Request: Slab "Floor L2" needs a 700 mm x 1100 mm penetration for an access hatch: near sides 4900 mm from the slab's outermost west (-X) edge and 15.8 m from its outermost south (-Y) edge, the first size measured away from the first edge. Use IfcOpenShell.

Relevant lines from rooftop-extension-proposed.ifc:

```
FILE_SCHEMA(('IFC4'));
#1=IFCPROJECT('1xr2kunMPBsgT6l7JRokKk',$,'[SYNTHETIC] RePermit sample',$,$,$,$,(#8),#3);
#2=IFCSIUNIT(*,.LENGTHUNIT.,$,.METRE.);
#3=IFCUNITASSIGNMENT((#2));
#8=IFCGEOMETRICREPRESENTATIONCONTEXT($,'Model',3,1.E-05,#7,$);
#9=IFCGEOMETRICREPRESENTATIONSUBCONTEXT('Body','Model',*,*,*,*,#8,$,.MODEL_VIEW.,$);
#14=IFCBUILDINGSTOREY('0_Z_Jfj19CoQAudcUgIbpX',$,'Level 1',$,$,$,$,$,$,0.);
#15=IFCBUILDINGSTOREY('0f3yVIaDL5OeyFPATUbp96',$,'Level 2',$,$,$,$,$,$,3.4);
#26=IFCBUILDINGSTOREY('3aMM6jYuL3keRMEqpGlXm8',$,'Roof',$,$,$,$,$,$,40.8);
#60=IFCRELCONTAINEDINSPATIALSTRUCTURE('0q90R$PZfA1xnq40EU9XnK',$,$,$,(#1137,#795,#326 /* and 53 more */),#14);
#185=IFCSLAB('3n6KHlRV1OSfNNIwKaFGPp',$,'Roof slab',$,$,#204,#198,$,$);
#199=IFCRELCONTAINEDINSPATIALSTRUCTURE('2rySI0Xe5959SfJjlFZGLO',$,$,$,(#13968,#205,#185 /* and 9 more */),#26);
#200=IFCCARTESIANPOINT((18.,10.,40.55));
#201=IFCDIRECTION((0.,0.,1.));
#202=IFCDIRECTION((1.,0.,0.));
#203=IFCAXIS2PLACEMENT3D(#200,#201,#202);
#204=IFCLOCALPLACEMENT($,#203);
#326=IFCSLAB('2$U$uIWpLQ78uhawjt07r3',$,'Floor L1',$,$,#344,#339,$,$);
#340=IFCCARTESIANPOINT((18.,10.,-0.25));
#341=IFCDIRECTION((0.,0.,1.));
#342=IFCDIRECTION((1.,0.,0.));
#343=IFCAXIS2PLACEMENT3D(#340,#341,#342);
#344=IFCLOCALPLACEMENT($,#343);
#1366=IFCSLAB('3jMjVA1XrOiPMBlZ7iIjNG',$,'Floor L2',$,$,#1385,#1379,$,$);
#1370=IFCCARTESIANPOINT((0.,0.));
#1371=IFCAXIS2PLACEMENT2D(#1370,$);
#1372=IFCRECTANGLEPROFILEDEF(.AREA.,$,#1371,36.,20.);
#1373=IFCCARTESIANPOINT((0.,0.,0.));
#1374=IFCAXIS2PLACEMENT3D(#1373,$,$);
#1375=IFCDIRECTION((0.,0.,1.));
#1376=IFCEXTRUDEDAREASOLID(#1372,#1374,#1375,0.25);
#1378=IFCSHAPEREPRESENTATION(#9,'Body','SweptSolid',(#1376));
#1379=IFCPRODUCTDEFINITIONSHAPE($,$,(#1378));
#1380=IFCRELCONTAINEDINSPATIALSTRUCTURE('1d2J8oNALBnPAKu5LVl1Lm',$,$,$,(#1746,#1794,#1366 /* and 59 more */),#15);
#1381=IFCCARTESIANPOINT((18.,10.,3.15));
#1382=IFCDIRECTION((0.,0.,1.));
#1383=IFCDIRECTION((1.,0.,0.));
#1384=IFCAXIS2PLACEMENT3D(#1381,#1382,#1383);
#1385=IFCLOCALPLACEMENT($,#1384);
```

```python
import numpy as np
import ifcopenshell
import ifcopenshell.api.feature
import ifcopenshell.api.geometry
import ifcopenshell.api.root
import ifcopenshell.geom
import ifcopenshell.util.placement
import ifcopenshell.util.representation
import ifcopenshell.util.shape
import ifcopenshell.util.unit

model = ifcopenshell.open("rooftop-extension-proposed.ifc")
unit_scale = ifcopenshell.util.unit.calculate_unit_scale(model)
settings = ifcopenshell.geom.settings()


def volume(element):
    """Net volume in cubic metres, openings subtracted."""
    shape = ifcopenshell.geom.create_shape(settings, element)
    return ifcopenshell.util.shape.get_volume(shape.geometry)


slab = model.by_guid("3jMjVA1XrOiPMBlZ7iIjNG")
before = volume(slab)

# Extent in the slab's own axes, in metres. The edges named are its -X and -Y sides.
slab_shape = ifcopenshell.geom.create_shape(settings, slab)
vertices = ifcopenshell.util.shape.get_vertices(slab_shape.geometry)
x_min, y_min, bottom = vertices.min(axis=0)
top = vertices[:, 2].max()

opening = ifcopenshell.api.root.create_entity(model, ifc_class="IfcOpeningElement", name="Access hatch opening", predefined_type="OPENING")
context = ifcopenshell.util.representation.get_context(model, "Model", "Body", "MODEL_VIEW")
width, depth = 0.7, 1.1
outline = [(0.0, 0.0), (width, 0.0), (width, depth), (0.0, depth), (0.0, 0.0)]
# Overshoot both faces by 50 mm so the cut is clean.
shape = ifcopenshell.api.geometry.add_slab_representation(
    model, context=context, depth=top - bottom + 0.1, polyline=outline
)
ifcopenshell.api.geometry.assign_representation(model, product=opening, representation=shape)

matrix = ifcopenshell.util.placement.get_local_placement(slab.ObjectPlacement)
matrix[:, 3] = matrix @ np.append(np.array([x_min + 4.9, y_min + 15.8, bottom - 0.05]) / unit_scale, 1.0)
ifcopenshell.api.geometry.edit_object_placement(model, product=opening, matrix=matrix, is_si=False)
ifcopenshell.api.feature.add_feature(model, feature=opening, element=slab)

after = volume(slab)

print(f"slab volume {before:.3f} -> {after:.3f} m3")

model.write("rooftop-extension-proposed_edited.ifc")
```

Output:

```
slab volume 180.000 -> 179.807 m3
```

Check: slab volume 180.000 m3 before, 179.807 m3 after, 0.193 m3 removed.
